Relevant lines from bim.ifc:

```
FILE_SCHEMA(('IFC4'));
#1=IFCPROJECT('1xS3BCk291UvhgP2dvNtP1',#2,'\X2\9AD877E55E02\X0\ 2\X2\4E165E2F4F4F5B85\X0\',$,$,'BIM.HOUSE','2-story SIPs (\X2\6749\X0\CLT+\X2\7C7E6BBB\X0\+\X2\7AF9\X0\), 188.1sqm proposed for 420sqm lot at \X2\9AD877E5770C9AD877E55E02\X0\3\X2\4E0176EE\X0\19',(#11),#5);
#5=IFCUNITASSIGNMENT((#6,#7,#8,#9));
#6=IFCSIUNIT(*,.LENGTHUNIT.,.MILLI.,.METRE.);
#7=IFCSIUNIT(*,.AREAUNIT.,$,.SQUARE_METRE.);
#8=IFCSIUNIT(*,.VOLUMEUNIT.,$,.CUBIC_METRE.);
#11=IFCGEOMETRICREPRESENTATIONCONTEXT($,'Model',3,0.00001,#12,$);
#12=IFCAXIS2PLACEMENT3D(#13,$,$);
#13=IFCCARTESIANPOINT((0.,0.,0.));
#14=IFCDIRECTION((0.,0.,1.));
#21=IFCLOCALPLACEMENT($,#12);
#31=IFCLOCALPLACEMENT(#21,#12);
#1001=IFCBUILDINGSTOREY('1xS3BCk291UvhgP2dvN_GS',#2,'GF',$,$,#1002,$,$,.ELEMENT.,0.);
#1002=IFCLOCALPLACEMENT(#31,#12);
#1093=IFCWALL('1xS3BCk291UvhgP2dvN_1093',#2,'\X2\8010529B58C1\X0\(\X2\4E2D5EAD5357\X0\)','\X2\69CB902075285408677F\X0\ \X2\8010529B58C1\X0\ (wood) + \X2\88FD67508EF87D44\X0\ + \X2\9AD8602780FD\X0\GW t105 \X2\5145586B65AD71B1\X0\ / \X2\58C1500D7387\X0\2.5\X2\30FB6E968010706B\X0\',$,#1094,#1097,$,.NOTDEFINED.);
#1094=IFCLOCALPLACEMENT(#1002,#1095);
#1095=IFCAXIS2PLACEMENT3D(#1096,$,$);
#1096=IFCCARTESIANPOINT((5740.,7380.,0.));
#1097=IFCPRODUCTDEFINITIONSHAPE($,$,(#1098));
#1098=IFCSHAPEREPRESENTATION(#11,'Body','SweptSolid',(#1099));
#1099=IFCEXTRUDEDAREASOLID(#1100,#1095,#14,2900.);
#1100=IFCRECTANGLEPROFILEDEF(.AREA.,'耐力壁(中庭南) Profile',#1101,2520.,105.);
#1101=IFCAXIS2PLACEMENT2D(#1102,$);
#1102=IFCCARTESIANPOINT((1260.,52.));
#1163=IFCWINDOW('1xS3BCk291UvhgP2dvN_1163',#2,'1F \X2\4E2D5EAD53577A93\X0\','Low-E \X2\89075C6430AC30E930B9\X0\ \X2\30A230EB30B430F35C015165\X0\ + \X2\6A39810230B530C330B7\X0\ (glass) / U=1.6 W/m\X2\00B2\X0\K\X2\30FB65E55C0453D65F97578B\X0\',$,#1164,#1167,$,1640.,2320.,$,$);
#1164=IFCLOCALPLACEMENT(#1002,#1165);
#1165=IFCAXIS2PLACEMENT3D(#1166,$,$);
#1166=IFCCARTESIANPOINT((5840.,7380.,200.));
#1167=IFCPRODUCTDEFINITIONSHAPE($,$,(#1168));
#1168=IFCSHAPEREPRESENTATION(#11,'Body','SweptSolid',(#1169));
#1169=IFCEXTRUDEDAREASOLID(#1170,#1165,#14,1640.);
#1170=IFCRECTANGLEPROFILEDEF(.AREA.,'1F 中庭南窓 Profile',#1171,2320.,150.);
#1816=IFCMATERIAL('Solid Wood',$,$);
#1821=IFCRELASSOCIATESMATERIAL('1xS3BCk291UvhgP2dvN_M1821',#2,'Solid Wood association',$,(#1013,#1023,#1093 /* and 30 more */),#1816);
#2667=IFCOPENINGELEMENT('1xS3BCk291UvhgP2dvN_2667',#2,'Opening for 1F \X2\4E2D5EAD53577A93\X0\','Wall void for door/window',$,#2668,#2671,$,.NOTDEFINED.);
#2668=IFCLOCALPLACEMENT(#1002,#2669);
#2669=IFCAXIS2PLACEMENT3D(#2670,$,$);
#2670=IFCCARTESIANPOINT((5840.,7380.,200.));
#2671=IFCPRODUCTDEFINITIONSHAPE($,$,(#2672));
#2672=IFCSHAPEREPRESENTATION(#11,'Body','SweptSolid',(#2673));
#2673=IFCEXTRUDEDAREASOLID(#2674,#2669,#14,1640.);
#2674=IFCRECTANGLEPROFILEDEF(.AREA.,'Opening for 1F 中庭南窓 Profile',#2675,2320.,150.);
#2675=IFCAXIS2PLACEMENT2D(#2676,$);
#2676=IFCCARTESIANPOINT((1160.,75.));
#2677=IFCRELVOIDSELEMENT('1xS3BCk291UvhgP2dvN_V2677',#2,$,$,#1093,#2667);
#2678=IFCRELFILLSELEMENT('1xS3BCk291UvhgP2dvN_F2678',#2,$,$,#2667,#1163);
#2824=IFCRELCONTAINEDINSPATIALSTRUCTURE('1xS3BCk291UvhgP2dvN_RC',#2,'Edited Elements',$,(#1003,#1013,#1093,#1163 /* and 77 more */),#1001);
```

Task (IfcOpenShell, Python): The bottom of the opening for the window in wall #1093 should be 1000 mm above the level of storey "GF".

```python
import numpy as np
import ifcopenshell
import ifcopenshell.api.geometry
import ifcopenshell.geom
import ifcopenshell.util.element
import ifcopenshell.util.placement
import ifcopenshell.util.shape
import ifcopenshell.util.unit

model = ifcopenshell.open("bim.ifc")
unit_scale = ifcopenshell.util.unit.calculate_unit_scale(model)

window = model.by_guid("1xS3BCk291UvhgP2dvN_1163")
opening = window.FillsVoids[0].RelatingOpeningElement
storey = ifcopenshell.util.element.get_container(window, ifc_class="IfcBuildingStorey")
level = ifcopenshell.util.placement.get_local_placement(storey.ObjectPlacement)[2, 3]

# The opening's origin need not be at the sill, so measure its lowest point.
shape = ifcopenshell.geom.create_shape(ifcopenshell.geom.settings(), opening)
bottom = ifcopenshell.util.shape.get_shape_bottom_elevation(shape, shape.geometry) / unit_scale
dz = level + 1000.0 - bottom

shift = np.array([0.0, 0.0, dz])
# The window is not placed relative to its opening, so move both.
for product in (opening, window):
    matrix = ifcopenshell.util.placement.get_local_placement(product.ObjectPlacement)
    matrix[:3, 3] += shift
    ifcopenshell.api.geometry.edit_object_placement(model, product=product, matrix=matrix, is_si=False)

print(f"moved by {dz * unit_scale:+.3f} m")

model.write("bim-out.ifc")
```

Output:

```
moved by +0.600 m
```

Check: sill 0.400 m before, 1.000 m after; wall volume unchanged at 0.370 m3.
